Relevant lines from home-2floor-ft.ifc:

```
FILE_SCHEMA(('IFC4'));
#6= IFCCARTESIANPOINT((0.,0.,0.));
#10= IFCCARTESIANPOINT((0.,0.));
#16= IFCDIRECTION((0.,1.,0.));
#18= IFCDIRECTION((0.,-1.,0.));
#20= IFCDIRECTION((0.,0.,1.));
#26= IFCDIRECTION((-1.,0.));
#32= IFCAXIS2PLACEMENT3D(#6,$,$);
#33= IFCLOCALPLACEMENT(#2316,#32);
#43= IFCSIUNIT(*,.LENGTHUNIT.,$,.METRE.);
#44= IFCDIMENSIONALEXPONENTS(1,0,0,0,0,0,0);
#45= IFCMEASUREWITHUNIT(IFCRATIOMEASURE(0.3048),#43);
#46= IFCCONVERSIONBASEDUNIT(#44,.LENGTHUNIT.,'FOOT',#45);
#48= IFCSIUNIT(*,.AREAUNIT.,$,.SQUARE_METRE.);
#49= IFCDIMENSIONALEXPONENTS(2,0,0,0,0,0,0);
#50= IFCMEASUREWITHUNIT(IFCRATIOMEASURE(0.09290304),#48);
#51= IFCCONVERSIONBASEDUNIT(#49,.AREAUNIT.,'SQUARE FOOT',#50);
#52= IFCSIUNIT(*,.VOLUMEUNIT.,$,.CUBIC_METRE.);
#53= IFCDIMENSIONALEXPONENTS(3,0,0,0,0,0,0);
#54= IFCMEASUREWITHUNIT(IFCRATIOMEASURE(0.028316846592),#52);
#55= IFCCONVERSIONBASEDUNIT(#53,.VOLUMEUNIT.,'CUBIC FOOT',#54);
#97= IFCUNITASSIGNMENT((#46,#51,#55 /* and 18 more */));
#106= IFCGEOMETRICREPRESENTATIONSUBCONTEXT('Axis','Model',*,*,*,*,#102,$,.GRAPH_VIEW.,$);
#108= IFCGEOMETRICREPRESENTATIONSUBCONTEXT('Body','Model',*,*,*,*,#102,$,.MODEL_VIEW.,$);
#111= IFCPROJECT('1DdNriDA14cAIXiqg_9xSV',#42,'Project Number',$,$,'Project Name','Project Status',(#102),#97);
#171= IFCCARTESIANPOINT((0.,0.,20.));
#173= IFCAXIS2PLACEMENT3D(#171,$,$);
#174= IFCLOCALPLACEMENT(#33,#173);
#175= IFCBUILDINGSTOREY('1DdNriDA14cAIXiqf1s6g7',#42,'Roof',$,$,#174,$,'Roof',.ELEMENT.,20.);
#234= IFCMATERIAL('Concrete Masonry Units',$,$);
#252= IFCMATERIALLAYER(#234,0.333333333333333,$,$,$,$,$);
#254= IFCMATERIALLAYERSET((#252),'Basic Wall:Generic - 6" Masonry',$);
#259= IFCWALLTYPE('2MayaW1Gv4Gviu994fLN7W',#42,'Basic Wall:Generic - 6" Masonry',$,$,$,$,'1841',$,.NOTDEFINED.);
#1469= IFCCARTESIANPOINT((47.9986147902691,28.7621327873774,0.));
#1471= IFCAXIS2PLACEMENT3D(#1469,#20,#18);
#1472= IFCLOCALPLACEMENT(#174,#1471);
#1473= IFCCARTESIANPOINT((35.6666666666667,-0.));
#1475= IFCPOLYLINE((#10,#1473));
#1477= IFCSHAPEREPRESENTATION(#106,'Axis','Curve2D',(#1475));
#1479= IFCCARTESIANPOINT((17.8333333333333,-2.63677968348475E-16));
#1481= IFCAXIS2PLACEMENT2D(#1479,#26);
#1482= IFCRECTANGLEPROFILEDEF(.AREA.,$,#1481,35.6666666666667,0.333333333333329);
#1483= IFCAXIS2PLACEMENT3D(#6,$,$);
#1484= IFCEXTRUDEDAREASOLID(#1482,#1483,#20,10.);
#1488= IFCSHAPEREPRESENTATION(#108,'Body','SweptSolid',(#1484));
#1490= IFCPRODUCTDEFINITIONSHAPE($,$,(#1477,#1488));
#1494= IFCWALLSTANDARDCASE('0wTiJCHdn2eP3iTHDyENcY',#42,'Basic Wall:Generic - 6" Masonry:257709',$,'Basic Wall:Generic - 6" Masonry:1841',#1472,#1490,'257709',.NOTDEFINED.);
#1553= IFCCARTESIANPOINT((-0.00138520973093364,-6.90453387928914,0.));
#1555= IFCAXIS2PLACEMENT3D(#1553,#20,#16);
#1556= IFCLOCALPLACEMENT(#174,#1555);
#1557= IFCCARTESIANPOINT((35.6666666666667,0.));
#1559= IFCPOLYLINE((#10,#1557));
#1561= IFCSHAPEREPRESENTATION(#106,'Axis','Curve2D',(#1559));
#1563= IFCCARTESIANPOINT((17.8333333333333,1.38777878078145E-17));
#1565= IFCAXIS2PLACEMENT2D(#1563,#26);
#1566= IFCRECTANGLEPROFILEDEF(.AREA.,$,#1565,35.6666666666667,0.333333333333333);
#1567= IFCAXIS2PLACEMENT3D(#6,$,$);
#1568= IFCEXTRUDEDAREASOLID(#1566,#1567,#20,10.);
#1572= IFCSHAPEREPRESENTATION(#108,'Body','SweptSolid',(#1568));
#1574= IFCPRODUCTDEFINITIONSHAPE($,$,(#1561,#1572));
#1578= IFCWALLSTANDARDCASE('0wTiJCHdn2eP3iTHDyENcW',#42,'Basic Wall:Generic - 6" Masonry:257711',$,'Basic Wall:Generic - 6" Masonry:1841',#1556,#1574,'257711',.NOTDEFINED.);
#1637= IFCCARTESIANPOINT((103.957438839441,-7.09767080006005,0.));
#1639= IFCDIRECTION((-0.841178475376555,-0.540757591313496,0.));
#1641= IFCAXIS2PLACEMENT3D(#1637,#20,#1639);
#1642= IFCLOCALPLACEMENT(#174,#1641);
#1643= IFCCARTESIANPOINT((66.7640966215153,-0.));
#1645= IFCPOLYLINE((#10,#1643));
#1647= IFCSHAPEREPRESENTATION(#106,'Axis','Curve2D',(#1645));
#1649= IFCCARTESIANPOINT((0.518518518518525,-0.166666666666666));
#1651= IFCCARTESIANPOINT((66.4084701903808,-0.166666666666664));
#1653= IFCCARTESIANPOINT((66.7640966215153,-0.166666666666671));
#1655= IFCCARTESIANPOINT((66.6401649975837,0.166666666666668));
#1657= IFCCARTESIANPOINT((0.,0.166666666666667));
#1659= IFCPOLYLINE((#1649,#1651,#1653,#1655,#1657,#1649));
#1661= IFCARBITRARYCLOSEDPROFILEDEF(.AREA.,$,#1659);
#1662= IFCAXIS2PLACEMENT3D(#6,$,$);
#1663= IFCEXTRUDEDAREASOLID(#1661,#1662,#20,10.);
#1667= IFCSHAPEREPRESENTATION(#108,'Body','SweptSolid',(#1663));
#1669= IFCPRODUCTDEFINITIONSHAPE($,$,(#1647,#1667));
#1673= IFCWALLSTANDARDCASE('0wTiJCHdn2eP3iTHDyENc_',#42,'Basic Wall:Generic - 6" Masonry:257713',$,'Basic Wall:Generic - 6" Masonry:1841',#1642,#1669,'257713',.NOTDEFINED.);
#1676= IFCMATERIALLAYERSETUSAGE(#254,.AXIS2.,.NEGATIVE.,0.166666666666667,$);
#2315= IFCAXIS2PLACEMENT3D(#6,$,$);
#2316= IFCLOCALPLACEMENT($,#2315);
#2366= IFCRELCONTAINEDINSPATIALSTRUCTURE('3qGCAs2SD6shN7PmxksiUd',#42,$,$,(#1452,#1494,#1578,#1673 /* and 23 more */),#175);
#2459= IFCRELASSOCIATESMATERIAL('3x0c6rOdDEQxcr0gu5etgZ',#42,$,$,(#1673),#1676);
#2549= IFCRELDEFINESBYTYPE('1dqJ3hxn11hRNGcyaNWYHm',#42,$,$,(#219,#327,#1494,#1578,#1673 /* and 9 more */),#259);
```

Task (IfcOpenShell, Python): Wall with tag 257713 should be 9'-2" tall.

```python
import ifcopenshell
import ifcopenshell.geom
import ifcopenshell.util.representation
import ifcopenshell.util.shape
import ifcopenshell.util.unit

model = ifcopenshell.open("home-2floor-ft.ifc")
unit_scale = ifcopenshell.util.unit.calculate_unit_scale(model)
settings = ifcopenshell.geom.settings()


def volume(element):
    """Net volume in cubic metres, openings subtracted."""
    shape = ifcopenshell.geom.create_shape(settings, element)
    return ifcopenshell.util.shape.get_volume(shape.geometry)


wall = model.by_guid("0wTiJCHdn2eP3iTHDyENc_")
before = volume(wall)

body = ifcopenshell.util.representation.get_representation(wall, "Model", "Body")
solid = body.Items[0]
old_height = solid.Depth
solid.Depth = 110 * 0.0254 / unit_scale
after = volume(wall)

print(f"height {old_height:g} -> {solid.Depth:g}, volume {before:.3f} -> {after:.3f} m3")

model.write("home-2floor-ft-out.ifc")
```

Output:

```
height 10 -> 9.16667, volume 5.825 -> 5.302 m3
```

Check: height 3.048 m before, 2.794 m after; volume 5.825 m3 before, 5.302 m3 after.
